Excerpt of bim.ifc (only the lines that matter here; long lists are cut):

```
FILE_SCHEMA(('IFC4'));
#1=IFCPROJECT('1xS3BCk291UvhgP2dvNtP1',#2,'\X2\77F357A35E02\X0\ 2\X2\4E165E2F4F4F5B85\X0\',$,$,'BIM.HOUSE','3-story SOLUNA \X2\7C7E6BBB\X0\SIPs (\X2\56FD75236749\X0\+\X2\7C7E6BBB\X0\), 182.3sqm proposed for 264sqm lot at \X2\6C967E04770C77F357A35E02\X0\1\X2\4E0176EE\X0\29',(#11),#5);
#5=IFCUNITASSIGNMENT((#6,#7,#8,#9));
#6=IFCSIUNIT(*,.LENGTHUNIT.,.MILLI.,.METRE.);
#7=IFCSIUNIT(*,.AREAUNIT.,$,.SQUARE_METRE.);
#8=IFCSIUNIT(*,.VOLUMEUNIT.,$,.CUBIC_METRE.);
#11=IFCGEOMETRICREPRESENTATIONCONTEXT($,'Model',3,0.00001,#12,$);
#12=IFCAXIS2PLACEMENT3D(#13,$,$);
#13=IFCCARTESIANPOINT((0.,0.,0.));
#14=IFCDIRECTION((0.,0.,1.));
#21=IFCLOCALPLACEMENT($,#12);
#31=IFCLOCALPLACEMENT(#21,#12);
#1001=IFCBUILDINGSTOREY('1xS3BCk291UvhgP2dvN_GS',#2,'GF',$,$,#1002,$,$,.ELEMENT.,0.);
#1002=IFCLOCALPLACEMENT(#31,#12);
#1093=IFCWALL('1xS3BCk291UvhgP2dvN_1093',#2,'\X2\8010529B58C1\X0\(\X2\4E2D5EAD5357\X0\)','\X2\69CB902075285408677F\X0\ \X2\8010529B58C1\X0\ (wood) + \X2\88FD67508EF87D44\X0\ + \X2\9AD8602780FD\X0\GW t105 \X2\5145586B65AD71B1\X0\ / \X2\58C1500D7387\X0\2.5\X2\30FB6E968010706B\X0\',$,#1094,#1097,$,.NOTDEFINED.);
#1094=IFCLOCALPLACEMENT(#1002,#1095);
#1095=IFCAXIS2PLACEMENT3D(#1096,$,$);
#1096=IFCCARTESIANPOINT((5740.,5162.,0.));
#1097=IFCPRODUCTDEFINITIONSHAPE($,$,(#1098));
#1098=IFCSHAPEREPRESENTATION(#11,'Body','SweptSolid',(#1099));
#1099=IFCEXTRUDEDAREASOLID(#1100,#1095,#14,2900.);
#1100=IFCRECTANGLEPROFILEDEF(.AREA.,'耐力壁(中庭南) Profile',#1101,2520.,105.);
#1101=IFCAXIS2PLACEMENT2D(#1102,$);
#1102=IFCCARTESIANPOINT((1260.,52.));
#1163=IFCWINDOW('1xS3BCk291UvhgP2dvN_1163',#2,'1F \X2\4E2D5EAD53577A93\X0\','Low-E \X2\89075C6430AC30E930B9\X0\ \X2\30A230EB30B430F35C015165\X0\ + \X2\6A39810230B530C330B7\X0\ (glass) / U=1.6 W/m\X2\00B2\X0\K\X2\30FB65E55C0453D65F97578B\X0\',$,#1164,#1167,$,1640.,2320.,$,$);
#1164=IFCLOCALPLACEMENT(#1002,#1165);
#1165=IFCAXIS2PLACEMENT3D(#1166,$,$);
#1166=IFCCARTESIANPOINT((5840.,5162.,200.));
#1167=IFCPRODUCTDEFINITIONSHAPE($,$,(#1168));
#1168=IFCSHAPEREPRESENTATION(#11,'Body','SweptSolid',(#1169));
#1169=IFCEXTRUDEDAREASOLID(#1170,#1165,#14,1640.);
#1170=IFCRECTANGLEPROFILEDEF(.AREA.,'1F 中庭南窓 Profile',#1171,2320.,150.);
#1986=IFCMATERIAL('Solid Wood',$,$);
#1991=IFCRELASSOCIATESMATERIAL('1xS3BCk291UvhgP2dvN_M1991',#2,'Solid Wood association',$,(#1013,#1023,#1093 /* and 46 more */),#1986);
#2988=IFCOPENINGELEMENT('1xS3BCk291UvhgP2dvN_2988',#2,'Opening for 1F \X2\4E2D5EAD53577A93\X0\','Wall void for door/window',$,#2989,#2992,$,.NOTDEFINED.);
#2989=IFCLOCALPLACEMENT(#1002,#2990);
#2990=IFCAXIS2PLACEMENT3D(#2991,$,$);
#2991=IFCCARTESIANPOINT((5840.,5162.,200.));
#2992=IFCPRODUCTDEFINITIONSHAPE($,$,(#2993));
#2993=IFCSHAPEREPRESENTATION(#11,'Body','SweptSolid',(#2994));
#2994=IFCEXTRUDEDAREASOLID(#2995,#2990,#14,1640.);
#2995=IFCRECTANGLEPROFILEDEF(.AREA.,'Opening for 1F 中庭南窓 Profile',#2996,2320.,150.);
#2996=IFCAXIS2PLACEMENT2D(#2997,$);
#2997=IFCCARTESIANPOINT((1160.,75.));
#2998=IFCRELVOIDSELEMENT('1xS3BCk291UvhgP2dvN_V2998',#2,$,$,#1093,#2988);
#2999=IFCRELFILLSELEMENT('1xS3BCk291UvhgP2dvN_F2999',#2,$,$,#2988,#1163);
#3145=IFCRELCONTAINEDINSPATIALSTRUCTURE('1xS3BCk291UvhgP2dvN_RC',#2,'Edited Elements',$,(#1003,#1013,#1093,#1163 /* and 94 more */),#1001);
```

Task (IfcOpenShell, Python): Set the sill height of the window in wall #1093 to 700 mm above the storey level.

```python
import numpy as np
import ifcopenshell
import ifcopenshell.api.geometry
import ifcopenshell.geom
import ifcopenshell.util.element
import ifcopenshell.util.placement
import ifcopenshell.util.shape
import ifcopenshell.util.unit

model = ifcopenshell.open("bim.ifc")
unit_scale = ifcopenshell.util.unit.calculate_unit_scale(model)

window = model.by_id(1163)
opening = window.FillsVoids[0].RelatingOpeningElement
storey = ifcopenshell.util.element.get_container(window, ifc_class="IfcBuildingStorey")
level = ifcopenshell.util.placement.get_local_placement(storey.ObjectPlacement)[2, 3]

# The opening's origin need not be at the sill, so measure its lowest point.
shape = ifcopenshell.geom.create_shape(ifcopenshell.geom.settings(), opening)
bottom = ifcopenshell.util.shape.get_shape_bottom_elevation(shape, shape.geometry) / unit_scale
dz = level + 0.7 / unit_scale - bottom

shift = np.array([0.0, 0.0, dz])
# The window is not placed relative to its opening, so move both.
for product in (opening, window):
    matrix = ifcopenshell.util.placement.get_local_placement(product.ObjectPlacement)
    matrix[:3, 3] += shift
    ifcopenshell.api.geometry.edit_object_placement(model, product=product, matrix=matrix, is_si=False)

print(f"moved by {dz * unit_scale:+.3f} m")

model.write("bim_rev.ifc")
```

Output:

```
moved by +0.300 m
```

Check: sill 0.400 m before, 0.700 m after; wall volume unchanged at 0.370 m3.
